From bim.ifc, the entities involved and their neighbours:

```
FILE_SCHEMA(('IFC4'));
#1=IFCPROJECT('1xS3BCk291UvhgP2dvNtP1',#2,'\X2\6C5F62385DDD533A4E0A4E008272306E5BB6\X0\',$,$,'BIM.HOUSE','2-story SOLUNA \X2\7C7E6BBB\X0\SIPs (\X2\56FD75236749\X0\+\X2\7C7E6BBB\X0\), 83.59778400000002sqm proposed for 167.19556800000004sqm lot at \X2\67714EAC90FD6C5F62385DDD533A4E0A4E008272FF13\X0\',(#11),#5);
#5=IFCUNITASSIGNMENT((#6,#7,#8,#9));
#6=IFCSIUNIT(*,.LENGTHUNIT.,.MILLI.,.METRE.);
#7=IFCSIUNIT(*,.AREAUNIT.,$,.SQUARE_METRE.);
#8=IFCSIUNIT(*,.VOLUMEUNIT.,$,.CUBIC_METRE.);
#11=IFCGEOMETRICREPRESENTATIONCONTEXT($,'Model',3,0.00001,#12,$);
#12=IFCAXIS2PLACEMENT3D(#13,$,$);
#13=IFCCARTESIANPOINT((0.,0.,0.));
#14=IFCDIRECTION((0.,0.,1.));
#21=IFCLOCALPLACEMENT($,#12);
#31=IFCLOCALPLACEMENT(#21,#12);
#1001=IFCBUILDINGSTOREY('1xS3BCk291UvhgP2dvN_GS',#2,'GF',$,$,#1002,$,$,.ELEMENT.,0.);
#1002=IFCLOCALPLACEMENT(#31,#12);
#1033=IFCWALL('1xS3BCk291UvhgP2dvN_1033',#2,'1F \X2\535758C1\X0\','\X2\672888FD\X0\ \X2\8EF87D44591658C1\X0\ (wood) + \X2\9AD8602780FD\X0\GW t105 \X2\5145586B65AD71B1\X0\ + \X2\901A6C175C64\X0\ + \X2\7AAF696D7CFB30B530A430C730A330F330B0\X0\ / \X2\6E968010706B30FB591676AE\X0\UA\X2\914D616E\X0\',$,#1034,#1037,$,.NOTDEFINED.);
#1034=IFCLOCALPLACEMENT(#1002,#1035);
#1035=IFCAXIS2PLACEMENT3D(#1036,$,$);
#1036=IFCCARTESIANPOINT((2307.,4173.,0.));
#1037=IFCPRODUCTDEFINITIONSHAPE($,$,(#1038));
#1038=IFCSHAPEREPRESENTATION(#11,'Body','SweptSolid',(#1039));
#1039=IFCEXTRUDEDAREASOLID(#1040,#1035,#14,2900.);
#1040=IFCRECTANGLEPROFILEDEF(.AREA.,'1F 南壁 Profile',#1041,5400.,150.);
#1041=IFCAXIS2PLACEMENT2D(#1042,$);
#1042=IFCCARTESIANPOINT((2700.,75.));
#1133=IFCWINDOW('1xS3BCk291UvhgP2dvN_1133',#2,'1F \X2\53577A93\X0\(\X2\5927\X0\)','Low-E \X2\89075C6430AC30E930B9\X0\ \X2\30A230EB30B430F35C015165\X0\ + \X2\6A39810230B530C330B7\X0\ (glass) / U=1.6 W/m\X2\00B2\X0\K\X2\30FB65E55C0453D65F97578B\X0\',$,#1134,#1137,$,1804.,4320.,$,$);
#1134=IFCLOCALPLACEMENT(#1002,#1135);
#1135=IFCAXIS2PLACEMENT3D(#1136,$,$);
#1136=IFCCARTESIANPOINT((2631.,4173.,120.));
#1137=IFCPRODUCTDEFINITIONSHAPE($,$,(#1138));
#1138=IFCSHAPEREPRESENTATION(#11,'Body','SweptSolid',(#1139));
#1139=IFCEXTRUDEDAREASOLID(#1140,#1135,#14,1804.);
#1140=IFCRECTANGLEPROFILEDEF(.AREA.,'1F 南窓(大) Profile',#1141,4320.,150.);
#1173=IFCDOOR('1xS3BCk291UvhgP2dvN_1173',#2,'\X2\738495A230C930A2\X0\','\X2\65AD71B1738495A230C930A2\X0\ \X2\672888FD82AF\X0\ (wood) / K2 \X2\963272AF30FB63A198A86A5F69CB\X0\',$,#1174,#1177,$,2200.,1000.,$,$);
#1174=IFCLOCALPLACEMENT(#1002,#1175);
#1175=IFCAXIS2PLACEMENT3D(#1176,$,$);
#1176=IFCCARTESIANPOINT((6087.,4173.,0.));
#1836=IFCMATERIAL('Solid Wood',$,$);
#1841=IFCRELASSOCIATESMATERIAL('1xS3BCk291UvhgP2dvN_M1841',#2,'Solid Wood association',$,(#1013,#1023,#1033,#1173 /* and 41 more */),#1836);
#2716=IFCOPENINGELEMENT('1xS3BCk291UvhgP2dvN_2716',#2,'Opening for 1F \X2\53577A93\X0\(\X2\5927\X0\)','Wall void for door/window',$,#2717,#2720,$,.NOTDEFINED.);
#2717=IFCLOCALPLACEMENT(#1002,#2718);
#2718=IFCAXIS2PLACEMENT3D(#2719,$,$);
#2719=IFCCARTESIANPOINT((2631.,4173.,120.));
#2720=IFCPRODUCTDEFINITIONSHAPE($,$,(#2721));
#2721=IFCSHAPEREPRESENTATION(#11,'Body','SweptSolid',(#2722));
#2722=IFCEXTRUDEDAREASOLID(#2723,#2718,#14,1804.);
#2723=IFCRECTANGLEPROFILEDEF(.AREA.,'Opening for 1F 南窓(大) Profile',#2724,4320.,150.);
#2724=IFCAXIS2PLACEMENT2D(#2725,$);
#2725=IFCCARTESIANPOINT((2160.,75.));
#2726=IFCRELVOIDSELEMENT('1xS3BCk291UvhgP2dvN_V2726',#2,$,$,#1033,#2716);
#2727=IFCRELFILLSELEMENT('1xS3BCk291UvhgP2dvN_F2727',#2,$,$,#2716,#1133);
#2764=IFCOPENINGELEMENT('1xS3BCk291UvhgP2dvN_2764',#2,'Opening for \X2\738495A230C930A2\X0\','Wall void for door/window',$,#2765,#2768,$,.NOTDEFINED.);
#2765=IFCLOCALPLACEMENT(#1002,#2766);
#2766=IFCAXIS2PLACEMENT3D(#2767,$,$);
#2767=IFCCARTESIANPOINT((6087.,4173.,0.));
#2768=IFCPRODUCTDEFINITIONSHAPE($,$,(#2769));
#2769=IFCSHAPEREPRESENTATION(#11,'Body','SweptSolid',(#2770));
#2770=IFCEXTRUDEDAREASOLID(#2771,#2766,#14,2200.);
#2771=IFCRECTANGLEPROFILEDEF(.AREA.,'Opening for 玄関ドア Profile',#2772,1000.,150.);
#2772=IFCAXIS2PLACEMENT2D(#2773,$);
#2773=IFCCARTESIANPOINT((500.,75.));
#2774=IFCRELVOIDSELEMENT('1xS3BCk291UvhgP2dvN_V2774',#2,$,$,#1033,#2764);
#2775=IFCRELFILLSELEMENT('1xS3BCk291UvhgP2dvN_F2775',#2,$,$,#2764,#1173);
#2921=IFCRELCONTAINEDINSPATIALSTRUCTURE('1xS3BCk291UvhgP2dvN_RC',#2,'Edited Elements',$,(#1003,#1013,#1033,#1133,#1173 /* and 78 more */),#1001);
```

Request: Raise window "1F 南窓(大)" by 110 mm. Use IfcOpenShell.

```python
import numpy as np
import ifcopenshell
import ifcopenshell.api.geometry
import ifcopenshell.util.placement
import ifcopenshell.util.unit

model = ifcopenshell.open("bim.ifc")
unit_scale = ifcopenshell.util.unit.calculate_unit_scale(model)

window = model.by_id(1133)
opening = window.FillsVoids[0].RelatingOpeningElement
dz = 110.0

shift = np.array([0.0, 0.0, dz])
# The window is not placed relative to its opening, so move both.
for product in (opening, window):
    matrix = ifcopenshell.util.placement.get_local_placement(product.ObjectPlacement)
    matrix[:3, 3] += shift
    ifcopenshell.api.geometry.edit_object_placement(model, product=product, matrix=matrix, is_si=False)

print(f"moved by {dz * unit_scale:+.3f} m")

model.write("bim-out.ifc")
```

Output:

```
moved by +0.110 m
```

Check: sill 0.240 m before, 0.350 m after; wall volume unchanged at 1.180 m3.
